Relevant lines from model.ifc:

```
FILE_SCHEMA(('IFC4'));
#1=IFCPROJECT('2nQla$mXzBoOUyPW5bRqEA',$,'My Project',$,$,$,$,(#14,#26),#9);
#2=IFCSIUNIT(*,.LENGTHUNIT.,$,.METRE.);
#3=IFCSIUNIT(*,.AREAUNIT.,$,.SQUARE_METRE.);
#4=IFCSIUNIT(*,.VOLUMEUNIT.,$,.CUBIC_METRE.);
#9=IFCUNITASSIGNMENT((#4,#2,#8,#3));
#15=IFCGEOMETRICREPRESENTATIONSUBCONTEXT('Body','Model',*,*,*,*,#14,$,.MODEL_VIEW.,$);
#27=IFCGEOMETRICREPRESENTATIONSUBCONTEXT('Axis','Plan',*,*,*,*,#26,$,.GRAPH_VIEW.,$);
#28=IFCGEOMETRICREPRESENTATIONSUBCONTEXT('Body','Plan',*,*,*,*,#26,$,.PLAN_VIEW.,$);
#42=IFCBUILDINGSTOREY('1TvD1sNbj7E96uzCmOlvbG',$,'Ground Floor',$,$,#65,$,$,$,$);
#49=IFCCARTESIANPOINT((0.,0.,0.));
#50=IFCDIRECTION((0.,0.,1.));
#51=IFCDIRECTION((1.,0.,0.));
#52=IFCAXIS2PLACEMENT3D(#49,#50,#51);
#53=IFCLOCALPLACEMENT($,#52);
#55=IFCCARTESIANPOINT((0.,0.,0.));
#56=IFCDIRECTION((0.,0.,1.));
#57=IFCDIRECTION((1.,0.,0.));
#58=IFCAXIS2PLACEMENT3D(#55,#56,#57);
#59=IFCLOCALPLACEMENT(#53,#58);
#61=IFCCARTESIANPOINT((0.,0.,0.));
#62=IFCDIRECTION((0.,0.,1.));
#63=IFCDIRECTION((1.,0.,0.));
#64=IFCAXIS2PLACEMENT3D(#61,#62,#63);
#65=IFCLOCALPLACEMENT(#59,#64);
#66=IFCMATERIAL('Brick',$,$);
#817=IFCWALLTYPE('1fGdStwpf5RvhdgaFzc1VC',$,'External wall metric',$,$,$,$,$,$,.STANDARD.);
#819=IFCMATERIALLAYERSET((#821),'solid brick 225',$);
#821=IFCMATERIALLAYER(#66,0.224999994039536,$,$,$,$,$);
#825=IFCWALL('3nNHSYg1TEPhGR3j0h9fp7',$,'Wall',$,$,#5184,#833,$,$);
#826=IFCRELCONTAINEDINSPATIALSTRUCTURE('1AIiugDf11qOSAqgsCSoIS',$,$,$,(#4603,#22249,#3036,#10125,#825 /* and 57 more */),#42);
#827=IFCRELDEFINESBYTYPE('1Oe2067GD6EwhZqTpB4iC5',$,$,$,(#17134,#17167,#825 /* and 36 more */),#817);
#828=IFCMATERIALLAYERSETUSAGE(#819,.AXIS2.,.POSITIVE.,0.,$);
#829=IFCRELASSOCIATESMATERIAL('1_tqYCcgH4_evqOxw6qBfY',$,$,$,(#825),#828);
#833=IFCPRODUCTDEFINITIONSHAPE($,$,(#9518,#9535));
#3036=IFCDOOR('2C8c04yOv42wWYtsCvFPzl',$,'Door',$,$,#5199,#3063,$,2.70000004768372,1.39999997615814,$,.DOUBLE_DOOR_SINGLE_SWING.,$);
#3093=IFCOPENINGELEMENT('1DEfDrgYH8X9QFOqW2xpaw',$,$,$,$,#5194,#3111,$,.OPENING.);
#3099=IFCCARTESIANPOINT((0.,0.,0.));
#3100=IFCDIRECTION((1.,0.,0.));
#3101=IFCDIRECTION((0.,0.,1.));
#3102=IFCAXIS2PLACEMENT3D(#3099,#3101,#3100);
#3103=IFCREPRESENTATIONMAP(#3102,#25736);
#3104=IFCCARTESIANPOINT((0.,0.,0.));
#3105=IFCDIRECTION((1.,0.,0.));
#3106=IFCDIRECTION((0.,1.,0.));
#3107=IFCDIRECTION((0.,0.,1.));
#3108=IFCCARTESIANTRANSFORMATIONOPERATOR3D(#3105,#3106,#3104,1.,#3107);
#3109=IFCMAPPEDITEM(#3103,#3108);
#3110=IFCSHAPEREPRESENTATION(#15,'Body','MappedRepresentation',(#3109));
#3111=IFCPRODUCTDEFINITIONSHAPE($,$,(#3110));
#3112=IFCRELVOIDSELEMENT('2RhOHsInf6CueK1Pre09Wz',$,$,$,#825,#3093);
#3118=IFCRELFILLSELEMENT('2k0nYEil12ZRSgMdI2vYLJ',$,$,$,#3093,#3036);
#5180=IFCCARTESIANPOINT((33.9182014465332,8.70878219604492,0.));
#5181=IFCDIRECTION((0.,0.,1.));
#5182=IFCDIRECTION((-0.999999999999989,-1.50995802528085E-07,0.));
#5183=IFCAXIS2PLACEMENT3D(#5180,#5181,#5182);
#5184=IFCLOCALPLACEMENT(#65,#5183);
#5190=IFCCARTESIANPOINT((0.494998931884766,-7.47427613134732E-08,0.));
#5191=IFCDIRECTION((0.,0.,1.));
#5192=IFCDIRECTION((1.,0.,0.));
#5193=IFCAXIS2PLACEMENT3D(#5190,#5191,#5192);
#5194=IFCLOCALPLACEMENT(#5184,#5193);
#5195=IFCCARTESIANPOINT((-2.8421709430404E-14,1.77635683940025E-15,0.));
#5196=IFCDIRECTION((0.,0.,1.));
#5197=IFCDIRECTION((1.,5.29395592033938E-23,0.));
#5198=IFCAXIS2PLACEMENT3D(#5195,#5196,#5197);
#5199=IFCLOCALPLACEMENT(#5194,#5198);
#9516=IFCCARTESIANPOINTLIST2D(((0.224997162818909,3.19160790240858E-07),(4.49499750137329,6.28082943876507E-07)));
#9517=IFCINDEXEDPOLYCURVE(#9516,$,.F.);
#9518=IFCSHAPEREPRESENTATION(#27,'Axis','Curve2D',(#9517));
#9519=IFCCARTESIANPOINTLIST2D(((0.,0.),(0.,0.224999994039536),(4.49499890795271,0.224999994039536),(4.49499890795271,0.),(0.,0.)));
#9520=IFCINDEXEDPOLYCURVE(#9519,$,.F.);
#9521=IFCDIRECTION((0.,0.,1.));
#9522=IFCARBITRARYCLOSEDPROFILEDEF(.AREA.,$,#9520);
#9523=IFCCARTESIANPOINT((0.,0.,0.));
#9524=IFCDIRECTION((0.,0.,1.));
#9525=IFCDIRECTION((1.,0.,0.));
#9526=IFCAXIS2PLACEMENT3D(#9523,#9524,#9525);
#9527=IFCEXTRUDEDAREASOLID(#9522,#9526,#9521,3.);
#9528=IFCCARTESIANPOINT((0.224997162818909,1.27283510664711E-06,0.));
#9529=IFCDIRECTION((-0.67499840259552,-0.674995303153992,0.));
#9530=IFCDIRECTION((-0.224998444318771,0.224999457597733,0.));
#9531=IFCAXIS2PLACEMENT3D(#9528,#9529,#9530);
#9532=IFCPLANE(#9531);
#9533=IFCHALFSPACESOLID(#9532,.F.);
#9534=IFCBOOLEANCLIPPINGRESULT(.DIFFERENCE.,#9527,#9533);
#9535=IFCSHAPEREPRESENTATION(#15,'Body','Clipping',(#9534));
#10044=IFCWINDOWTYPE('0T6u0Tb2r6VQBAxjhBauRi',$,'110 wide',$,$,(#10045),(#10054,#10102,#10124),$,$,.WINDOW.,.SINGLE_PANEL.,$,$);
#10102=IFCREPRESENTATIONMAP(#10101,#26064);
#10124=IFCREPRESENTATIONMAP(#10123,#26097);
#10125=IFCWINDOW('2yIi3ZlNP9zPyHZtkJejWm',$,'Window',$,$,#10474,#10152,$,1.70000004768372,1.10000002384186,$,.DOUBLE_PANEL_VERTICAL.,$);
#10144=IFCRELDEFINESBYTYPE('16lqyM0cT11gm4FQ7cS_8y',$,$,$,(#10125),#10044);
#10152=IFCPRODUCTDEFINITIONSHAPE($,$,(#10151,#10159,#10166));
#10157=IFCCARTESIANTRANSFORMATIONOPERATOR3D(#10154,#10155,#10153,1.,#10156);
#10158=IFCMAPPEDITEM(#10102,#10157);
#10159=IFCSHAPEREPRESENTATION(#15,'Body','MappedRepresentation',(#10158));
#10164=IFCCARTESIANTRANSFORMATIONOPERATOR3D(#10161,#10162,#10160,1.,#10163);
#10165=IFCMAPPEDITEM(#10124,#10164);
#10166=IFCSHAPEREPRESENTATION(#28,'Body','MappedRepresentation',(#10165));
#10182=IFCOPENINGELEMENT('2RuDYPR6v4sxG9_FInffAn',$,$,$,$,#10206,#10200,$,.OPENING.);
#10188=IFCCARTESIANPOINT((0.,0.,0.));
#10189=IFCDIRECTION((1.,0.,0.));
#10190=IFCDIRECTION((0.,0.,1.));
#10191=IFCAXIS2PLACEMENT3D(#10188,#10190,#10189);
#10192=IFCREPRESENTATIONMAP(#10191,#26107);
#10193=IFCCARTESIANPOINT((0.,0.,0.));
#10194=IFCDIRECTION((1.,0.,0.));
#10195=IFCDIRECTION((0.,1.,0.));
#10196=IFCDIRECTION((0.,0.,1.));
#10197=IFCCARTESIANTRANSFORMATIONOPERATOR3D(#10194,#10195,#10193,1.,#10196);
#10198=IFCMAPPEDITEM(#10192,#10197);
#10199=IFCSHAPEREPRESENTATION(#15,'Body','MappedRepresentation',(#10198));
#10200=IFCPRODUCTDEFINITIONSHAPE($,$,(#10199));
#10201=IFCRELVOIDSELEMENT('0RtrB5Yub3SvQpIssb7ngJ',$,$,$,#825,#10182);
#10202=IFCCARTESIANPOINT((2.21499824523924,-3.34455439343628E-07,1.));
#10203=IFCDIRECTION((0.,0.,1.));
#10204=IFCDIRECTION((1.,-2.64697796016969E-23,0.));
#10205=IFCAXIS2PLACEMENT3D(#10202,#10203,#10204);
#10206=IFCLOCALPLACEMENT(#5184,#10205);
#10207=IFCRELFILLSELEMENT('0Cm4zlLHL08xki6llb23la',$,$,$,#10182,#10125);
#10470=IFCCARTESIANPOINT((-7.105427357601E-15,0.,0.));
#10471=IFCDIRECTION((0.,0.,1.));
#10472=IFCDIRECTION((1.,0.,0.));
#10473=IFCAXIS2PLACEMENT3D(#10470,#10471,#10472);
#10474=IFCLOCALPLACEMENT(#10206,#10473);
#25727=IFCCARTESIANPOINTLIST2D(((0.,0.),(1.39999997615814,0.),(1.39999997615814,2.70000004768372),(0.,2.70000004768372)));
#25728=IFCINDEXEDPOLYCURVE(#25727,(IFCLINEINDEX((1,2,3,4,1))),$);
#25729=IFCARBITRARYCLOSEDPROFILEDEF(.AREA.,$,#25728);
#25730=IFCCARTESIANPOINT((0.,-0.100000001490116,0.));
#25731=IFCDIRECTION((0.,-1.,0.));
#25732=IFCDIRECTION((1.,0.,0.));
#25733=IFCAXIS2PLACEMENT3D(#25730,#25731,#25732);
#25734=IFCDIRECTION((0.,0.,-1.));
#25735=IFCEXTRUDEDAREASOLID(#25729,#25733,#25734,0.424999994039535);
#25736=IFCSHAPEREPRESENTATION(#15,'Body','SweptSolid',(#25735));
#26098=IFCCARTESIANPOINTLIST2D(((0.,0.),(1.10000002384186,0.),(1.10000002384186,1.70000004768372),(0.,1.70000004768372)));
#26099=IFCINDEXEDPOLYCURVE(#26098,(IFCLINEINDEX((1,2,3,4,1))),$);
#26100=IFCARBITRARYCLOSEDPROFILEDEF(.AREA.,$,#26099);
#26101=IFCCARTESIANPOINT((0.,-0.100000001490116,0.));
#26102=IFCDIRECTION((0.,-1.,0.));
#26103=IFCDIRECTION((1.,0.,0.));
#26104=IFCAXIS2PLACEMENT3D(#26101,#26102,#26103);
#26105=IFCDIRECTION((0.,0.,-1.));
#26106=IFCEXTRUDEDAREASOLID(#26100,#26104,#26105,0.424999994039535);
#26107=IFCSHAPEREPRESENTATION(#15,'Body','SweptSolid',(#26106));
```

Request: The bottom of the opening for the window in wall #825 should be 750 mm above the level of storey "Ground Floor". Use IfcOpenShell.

```python
import numpy as np
import ifcopenshell
import ifcopenshell.api.geometry
import ifcopenshell.geom
import ifcopenshell.util.element
import ifcopenshell.util.placement
import ifcopenshell.util.shape
import ifcopenshell.util.unit

model = ifcopenshell.open("model.ifc")
unit_scale = ifcopenshell.util.unit.calculate_unit_scale(model)

window = model.by_id(10125)
opening = window.FillsVoids[0].RelatingOpeningElement
storey = ifcopenshell.util.element.get_container(window, ifc_class="IfcBuildingStorey")
level = ifcopenshell.util.placement.get_local_placement(storey.ObjectPlacement)[2, 3]

# The opening's origin need not be at the sill, so measure its lowest point.
shape = ifcopenshell.geom.create_shape(ifcopenshell.geom.settings(), opening)
bottom = ifcopenshell.util.shape.get_shape_bottom_elevation(shape, shape.geometry) / unit_scale
dz = level + 0.75 / unit_scale - bottom

shift = np.array([0.0, 0.0, dz])
# The window is placed relative to its opening, so it follows when the opening moves.
matrix = ifcopenshell.util.placement.get_local_placement(opening.ObjectPlacement)
matrix[:3, 3] += shift
ifcopenshell.api.geometry.edit_object_placement(
    model, product=opening, matrix=matrix, is_si=False, should_transform_children=True
)

print(f"moved by {dz * unit_scale:+.3f} m")

model.write("model_edited.ifc")
```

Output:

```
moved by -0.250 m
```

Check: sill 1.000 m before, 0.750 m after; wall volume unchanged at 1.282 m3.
